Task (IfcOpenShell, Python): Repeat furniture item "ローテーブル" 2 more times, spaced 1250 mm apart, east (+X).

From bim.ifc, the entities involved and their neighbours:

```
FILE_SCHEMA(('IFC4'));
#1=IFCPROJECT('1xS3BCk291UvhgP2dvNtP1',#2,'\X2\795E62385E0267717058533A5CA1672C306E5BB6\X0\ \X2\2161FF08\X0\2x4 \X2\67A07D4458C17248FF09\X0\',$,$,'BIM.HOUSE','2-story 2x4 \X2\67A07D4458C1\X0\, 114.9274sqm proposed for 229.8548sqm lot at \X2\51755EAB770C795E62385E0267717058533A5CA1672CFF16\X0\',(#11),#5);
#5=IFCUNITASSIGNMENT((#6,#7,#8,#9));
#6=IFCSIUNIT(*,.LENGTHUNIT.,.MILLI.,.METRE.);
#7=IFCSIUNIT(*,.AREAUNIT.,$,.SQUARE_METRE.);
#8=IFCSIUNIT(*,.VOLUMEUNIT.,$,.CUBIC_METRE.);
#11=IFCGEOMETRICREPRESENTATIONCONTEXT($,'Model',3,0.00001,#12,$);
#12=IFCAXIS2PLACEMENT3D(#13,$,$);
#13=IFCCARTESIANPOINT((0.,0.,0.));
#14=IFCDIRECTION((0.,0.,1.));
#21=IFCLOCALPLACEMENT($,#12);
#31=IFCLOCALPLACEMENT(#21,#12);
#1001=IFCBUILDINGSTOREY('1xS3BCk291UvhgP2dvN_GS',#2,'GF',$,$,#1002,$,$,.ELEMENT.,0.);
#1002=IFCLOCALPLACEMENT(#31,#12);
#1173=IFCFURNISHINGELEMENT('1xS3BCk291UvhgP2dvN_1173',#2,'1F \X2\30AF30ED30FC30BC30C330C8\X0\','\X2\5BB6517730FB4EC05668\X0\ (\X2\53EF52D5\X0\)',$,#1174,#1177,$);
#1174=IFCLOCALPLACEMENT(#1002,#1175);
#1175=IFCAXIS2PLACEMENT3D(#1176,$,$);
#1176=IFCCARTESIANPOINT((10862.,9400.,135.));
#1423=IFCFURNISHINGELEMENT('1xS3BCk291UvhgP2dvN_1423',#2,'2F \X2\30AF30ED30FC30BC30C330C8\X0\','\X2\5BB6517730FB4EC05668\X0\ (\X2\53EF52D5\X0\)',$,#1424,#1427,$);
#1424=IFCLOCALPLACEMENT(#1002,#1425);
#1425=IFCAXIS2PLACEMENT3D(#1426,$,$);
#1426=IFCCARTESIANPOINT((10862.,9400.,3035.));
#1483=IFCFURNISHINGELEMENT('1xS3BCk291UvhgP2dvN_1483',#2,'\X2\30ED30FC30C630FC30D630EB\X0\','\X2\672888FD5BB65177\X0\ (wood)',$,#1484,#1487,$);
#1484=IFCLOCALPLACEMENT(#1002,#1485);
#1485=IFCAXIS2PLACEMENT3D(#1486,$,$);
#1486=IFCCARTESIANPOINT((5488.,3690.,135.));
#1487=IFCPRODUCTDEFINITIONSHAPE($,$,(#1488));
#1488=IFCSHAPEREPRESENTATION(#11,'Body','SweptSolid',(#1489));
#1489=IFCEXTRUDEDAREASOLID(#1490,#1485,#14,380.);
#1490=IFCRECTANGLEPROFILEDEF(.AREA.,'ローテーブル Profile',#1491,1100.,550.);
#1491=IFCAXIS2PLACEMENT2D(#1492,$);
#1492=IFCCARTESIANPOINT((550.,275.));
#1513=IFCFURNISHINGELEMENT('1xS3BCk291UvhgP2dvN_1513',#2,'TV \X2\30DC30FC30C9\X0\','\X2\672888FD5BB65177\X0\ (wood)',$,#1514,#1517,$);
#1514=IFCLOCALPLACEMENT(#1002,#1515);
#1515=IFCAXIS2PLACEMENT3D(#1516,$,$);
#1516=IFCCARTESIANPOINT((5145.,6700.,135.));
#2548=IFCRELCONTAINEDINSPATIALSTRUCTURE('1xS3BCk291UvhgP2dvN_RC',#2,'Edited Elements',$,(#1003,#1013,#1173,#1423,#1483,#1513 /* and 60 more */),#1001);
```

```python
import numpy as np
import ifcopenshell
import ifcopenshell.api.geometry
import ifcopenshell.api.root
import ifcopenshell.util.element
import ifcopenshell.util.placement
import ifcopenshell.util.unit

model = ifcopenshell.open("bim.ifc")
unit_scale = ifcopenshell.util.unit.calculate_unit_scale(model)


def reuse_history(source, copy):
    """copy_class also copies each property set's owner history, people and application; keep the originals."""
    for rel in copy.IsDefinedBy:
        if rel.is_a("IfcRelDefinesByProperties") and (history := rel.RelatingPropertyDefinition.OwnerHistory):
            rel.RelatingPropertyDefinition.OwnerHistory = source.OwnerHistory
            ifcopenshell.util.element.remove_deep2(model, history)


source = model.by_id(1483)
base = ifcopenshell.util.placement.get_local_placement(source.ObjectPlacement)
step = np.array([1.0, 0.0, 0.0]) * 1.25 / unit_scale

for i in range(1, 3):
    copy = ifcopenshell.api.root.copy_class(model, product=source)
    copy.Representation = ifcopenshell.util.element.copy_deep(
        model, source.Representation, exclude=["IfcGeometricRepresentationContext", "IfcRepresentationMap"]
    )
    reuse_history(source, copy)
    matrix = base.copy()
    matrix[:3, 3] += i * step
    print("added at", matrix[:3, 3].round(3) + 0.0)
    ifcopenshell.api.geometry.edit_object_placement(model, product=copy, matrix=matrix, is_si=False)

model.write("bim_edited.ifc")
```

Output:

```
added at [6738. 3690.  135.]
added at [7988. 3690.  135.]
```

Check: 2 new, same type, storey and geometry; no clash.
